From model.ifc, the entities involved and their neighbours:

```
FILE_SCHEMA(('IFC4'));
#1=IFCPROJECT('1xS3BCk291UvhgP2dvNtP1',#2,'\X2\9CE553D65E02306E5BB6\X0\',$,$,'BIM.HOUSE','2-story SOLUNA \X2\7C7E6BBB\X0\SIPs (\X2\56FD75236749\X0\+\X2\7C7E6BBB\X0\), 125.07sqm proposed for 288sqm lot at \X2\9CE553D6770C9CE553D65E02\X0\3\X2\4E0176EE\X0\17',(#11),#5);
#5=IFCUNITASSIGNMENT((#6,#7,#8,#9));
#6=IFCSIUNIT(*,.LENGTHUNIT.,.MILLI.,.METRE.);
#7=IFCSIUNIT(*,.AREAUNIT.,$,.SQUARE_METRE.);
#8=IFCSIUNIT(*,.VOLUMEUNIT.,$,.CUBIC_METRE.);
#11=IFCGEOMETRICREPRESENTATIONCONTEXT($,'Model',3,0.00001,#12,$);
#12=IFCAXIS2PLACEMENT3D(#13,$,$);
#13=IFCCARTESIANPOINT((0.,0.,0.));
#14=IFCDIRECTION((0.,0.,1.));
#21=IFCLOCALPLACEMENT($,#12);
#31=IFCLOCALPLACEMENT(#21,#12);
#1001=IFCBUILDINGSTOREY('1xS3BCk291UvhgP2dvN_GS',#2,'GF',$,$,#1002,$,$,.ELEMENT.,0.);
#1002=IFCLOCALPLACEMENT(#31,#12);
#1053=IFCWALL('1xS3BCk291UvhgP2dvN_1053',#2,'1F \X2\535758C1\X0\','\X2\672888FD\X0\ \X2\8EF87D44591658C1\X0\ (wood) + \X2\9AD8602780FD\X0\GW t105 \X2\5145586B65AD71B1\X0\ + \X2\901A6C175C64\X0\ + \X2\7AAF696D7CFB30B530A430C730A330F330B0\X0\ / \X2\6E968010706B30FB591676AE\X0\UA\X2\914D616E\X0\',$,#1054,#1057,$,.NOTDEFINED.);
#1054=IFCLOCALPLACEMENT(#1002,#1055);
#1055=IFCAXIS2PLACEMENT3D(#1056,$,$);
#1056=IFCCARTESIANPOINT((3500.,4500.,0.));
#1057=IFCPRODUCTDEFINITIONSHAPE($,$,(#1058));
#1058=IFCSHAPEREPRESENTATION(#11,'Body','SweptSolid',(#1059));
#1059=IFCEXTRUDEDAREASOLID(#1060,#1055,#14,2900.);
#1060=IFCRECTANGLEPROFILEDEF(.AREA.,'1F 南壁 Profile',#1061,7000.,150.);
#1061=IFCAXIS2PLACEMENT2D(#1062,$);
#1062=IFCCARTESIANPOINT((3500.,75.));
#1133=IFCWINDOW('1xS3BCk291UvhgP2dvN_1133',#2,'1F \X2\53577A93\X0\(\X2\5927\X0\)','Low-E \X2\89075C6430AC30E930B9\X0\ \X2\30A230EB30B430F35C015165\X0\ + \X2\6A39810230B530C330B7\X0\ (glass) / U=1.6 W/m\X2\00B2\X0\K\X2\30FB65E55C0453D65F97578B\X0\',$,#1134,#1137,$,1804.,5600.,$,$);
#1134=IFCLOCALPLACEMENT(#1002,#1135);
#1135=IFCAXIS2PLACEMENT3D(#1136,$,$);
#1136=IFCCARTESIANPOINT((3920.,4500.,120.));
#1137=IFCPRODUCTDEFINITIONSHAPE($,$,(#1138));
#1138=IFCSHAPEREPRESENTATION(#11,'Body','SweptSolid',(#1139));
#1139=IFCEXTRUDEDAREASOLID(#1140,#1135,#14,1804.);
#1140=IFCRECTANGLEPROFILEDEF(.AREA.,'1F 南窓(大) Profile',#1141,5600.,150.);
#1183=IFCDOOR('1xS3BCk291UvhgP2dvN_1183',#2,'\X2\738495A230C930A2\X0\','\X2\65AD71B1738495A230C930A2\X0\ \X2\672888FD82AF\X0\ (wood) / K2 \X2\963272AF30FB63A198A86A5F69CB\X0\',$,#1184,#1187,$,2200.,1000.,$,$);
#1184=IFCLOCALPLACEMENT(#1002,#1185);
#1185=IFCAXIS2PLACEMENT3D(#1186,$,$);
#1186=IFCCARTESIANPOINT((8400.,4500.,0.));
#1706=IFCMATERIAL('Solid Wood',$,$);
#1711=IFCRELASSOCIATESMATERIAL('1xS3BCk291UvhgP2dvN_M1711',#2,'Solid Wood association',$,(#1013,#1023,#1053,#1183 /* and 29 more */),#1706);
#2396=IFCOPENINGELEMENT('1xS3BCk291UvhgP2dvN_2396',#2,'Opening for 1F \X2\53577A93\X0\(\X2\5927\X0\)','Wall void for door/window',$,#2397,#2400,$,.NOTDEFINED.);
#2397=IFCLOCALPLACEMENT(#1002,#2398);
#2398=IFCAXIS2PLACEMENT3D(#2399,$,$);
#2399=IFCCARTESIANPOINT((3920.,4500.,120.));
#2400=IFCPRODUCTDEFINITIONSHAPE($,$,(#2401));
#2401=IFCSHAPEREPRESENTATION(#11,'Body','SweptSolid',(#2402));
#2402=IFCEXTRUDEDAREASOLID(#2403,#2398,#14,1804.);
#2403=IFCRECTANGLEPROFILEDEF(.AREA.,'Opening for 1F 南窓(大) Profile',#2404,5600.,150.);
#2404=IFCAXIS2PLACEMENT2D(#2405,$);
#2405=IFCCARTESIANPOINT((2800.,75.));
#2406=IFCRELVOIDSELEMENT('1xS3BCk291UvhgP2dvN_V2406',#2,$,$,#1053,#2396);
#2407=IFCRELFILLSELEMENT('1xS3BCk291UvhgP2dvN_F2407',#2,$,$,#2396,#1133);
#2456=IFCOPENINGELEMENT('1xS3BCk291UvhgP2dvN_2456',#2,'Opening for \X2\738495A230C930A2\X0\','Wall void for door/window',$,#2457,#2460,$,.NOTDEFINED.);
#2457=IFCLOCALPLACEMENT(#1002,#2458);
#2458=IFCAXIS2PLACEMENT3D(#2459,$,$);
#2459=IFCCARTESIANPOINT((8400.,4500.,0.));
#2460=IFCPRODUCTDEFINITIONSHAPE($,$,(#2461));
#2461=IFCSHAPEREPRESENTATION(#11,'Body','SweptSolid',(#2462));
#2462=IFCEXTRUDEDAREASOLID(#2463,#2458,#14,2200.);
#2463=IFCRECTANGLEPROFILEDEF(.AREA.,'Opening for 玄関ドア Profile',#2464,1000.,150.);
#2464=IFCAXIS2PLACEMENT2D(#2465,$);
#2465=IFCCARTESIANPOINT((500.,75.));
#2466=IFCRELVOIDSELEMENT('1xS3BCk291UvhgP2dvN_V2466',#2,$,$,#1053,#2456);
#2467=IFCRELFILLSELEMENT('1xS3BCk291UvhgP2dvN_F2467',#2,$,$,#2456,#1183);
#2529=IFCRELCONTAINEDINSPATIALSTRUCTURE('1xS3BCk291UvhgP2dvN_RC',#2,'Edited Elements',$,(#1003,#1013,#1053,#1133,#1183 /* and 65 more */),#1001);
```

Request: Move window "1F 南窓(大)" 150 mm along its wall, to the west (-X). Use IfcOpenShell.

```python
import ifcopenshell
import ifcopenshell.api.geometry
import ifcopenshell.util.placement
import ifcopenshell.util.unit

model = ifcopenshell.open("model.ifc")
unit_scale = ifcopenshell.util.unit.calculate_unit_scale(model)

window = model.by_guid("1xS3BCk291UvhgP2dvN_1133")
opening = window.FillsVoids[0].RelatingOpeningElement
wall = opening.VoidsElements[0].RelatingBuildingElement

wall_matrix = ifcopenshell.util.placement.get_local_placement(wall.ObjectPlacement)
shift = wall_matrix[:3, 0] * -0.15 / unit_scale
before = ifcopenshell.util.placement.get_local_placement(window.ObjectPlacement)[:3, 3].copy()

# The window is not placed relative to its opening, so move both.
for product in (opening, window):
    matrix = ifcopenshell.util.placement.get_local_placement(product.ObjectPlacement)
    matrix[:3, 3] += shift
    ifcopenshell.api.geometry.edit_object_placement(model, product=product, matrix=matrix, is_si=False)

after = ifcopenshell.util.placement.get_local_placement(window.ObjectPlacement)[:3, 3]
print("window moved by", (after - before).round(3) + 0.0)

model.write("model_rev.ifc")
```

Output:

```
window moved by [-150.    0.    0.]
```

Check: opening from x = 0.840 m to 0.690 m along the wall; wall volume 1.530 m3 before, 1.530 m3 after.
